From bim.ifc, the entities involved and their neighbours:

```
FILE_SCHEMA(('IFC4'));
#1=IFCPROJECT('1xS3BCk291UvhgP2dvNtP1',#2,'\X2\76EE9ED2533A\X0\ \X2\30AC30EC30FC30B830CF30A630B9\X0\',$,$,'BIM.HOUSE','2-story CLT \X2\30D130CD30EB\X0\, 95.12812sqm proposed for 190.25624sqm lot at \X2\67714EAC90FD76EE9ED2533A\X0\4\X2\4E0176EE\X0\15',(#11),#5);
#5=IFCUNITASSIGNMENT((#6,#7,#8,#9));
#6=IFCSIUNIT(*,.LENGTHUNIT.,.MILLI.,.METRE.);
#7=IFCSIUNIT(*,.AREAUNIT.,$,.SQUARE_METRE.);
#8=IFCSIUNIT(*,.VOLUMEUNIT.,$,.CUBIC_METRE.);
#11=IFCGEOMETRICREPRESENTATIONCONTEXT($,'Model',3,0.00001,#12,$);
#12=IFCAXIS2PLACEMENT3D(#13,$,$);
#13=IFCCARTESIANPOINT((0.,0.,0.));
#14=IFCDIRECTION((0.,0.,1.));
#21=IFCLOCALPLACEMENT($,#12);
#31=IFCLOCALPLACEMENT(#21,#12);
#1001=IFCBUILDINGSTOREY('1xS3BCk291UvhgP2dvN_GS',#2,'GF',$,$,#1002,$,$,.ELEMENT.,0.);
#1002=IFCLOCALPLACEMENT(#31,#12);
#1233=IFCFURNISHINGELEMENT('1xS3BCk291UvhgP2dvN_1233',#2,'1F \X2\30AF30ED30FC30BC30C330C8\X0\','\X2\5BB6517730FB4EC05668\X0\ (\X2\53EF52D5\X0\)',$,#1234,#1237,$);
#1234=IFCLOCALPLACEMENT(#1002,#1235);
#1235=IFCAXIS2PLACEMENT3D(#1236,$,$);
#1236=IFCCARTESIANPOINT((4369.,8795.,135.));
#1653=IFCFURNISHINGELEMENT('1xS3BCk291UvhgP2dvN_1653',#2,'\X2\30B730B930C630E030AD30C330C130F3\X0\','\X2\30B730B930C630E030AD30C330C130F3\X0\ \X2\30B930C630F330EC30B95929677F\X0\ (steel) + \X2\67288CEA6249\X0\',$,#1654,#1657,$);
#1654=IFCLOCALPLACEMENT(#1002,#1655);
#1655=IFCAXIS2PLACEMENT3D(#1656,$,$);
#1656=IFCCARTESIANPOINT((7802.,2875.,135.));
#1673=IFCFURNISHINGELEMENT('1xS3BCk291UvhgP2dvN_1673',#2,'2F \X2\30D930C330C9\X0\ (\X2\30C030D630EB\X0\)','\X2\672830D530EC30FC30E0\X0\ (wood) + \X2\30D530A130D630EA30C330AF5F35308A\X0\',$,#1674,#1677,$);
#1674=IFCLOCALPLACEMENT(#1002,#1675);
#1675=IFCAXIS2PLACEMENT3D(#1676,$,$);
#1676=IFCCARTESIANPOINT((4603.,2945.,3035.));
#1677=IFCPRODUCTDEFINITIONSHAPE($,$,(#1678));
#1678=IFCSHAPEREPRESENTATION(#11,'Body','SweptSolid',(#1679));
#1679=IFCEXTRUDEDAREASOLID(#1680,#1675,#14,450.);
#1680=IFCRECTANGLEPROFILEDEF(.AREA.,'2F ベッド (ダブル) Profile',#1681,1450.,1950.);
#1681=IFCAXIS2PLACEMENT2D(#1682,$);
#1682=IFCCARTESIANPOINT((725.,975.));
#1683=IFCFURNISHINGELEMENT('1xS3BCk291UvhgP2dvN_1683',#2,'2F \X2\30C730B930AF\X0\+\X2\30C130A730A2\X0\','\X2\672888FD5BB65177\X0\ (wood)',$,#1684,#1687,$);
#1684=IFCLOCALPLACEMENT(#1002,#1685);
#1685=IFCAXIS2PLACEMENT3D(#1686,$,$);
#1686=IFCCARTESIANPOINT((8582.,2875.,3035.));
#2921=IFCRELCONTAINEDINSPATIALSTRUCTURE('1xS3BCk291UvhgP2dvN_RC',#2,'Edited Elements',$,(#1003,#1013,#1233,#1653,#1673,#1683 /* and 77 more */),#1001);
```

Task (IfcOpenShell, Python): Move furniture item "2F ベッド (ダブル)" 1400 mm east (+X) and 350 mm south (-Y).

```python
import ifcopenshell
import ifcopenshell.api.geometry
import ifcopenshell.util.placement

model = ifcopenshell.open("bim.ifc")

item = model.by_guid("1xS3BCk291UvhgP2dvN_1673")
matrix = ifcopenshell.util.placement.get_local_placement(item.ObjectPlacement)
matrix[0, 3] += 1400.0
matrix[1, 3] -= 350.0
ifcopenshell.api.geometry.edit_object_placement(model, product=item, matrix=matrix, is_si=False)

print(ifcopenshell.util.placement.get_local_placement(item.ObjectPlacement).round(3) + 0.0)

model.write("bim-out.ifc")
```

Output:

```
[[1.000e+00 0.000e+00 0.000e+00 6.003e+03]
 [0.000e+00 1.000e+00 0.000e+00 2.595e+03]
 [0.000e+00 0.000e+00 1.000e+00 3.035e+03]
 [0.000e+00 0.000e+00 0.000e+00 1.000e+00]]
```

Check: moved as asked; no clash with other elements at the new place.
